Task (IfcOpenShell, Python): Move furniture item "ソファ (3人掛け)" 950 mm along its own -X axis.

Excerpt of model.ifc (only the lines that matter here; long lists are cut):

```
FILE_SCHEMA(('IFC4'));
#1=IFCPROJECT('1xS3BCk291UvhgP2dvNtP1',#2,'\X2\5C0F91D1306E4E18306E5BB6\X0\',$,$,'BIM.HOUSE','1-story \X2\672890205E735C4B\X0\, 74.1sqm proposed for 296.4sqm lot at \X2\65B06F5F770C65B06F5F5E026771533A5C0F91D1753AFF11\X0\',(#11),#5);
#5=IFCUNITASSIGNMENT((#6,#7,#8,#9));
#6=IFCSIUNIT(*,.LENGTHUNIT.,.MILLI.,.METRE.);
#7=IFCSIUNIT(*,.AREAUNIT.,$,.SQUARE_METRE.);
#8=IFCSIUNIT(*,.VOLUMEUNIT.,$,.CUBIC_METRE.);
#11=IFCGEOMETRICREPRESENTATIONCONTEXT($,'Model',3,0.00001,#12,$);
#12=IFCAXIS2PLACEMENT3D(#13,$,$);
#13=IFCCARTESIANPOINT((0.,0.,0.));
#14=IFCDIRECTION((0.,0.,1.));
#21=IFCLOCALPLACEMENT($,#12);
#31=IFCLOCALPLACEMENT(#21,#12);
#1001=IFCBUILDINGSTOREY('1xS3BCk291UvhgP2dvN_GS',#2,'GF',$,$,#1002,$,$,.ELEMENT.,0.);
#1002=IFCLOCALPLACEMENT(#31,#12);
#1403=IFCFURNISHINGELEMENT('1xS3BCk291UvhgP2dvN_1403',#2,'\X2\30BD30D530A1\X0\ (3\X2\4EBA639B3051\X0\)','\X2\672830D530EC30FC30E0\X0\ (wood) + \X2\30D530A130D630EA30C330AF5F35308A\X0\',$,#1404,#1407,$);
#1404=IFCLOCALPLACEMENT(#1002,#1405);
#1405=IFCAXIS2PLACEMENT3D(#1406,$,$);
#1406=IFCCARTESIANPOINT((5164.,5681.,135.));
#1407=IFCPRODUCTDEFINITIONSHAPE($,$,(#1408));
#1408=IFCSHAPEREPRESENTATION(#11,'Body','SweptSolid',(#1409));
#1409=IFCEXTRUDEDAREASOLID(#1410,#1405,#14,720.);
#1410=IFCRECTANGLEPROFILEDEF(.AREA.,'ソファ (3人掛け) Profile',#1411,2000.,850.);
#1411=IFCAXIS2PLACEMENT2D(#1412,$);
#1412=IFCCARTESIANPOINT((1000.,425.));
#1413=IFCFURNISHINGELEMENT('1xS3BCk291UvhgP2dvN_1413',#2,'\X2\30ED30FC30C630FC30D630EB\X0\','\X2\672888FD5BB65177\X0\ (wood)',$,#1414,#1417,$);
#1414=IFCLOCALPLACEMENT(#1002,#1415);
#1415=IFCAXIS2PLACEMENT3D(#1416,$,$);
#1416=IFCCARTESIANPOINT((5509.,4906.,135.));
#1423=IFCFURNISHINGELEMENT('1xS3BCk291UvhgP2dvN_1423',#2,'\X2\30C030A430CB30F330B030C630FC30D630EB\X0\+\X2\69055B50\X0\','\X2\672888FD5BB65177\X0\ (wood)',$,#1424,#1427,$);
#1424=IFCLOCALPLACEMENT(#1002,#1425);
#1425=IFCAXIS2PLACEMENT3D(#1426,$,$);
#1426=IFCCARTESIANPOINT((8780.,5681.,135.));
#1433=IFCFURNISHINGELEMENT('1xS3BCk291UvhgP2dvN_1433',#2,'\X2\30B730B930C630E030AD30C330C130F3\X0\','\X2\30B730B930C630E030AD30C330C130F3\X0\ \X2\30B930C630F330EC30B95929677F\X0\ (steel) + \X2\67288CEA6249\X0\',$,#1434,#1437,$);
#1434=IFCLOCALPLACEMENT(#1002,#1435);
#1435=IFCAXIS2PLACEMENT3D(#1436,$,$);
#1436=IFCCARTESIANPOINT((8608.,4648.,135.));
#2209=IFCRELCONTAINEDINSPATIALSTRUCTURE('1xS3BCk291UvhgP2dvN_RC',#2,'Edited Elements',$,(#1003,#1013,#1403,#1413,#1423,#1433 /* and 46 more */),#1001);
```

```python
import ifcopenshell
import ifcopenshell.api.geometry
import ifcopenshell.util.placement
import ifcopenshell.util.unit

model = ifcopenshell.open("model.ifc")
unit_scale = ifcopenshell.util.unit.calculate_unit_scale(model)

item = model.by_id(1403)
matrix = ifcopenshell.util.placement.get_local_placement(item.ObjectPlacement)
matrix[:3, 3] -= matrix[:3, 0] * 0.95 / unit_scale
ifcopenshell.api.geometry.edit_object_placement(model, product=item, matrix=matrix, is_si=False)

print(ifcopenshell.util.placement.get_local_placement(item.ObjectPlacement).round(3) + 0.0)

model.write("model_v2.ifc")
```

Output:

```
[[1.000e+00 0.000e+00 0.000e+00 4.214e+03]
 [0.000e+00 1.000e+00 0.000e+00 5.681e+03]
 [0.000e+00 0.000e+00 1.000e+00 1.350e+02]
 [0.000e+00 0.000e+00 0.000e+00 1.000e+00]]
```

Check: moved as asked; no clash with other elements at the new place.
